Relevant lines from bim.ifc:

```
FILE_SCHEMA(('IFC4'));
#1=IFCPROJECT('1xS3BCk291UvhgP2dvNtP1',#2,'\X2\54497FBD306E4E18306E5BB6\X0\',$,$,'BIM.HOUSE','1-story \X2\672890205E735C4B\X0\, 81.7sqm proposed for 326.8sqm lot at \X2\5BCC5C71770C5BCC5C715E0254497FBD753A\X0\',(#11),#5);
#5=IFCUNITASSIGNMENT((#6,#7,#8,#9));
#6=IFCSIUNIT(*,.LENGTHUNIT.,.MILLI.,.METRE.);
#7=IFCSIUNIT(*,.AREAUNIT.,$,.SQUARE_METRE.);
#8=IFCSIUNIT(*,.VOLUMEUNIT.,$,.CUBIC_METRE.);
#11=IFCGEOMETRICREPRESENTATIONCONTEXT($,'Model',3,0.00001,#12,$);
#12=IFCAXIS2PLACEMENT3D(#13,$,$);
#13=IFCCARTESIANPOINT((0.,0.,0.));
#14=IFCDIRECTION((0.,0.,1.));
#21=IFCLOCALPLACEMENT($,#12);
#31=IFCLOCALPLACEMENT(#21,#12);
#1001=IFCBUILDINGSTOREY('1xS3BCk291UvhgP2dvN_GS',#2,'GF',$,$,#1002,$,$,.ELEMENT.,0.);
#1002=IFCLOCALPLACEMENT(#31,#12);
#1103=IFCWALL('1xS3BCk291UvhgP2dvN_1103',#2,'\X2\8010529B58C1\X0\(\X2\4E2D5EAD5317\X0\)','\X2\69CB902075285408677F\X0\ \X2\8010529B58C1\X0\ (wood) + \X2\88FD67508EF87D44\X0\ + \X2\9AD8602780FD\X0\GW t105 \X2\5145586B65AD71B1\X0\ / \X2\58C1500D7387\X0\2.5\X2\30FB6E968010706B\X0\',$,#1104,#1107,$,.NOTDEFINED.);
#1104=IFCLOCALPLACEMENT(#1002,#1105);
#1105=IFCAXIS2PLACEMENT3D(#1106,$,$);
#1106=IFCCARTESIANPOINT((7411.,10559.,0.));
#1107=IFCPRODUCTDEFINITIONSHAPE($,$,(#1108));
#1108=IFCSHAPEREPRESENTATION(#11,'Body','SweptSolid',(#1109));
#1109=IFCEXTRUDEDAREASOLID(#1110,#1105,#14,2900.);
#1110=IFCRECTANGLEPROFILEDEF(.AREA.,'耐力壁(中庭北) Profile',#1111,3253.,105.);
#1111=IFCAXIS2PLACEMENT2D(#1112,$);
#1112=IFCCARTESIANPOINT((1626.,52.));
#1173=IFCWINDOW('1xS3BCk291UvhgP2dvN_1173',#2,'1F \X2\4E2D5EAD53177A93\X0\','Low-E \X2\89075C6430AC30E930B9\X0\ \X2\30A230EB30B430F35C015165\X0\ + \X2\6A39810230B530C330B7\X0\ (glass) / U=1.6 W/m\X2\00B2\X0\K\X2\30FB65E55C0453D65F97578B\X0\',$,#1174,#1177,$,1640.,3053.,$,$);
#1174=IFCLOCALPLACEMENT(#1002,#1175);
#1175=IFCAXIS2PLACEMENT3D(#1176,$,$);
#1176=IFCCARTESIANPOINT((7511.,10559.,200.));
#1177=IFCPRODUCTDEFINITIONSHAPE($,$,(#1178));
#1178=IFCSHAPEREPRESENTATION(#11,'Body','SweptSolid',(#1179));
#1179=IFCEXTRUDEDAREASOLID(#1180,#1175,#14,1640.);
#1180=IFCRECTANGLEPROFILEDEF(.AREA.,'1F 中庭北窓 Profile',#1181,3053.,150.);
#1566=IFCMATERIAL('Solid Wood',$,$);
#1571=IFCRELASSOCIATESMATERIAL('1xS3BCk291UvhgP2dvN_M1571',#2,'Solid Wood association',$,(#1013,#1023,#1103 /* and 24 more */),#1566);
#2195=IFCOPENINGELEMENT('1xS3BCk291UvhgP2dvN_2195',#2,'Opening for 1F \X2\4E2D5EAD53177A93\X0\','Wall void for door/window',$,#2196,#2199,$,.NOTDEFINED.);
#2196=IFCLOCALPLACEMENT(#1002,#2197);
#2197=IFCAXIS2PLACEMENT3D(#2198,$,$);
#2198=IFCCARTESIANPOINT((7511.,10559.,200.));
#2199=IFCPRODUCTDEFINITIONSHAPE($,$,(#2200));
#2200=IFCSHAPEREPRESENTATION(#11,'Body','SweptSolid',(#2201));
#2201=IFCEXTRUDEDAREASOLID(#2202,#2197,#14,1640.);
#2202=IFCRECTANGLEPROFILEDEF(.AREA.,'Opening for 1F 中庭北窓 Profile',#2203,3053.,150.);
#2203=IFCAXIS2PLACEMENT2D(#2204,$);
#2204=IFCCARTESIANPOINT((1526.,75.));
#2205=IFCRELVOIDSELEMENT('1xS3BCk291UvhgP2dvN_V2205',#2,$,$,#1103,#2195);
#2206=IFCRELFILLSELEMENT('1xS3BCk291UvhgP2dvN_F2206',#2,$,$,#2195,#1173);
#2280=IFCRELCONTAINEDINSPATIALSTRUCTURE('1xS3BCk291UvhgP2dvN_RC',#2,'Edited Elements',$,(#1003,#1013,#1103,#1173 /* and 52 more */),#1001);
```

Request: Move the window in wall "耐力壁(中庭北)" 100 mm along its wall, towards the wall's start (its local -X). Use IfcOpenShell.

```python
import ifcopenshell
import ifcopenshell.api.geometry
import ifcopenshell.util.placement
import ifcopenshell.util.unit

model = ifcopenshell.open("bim.ifc")
unit_scale = ifcopenshell.util.unit.calculate_unit_scale(model)

window = model.by_guid("1xS3BCk291UvhgP2dvN_1173")
opening = window.FillsVoids[0].RelatingOpeningElement
wall = opening.VoidsElements[0].RelatingBuildingElement

wall_matrix = ifcopenshell.util.placement.get_local_placement(wall.ObjectPlacement)
shift = wall_matrix[:3, 0] * -0.1 / unit_scale
before = ifcopenshell.util.placement.get_local_placement(window.ObjectPlacement)[:3, 3].copy()

# The window is not placed relative to its opening, so move both.
for product in (opening, window):
    matrix = ifcopenshell.util.placement.get_local_placement(product.ObjectPlacement)
    matrix[:3, 3] += shift
    ifcopenshell.api.geometry.edit_object_placement(model, product=product, matrix=matrix, is_si=False)

after = ifcopenshell.util.placement.get_local_placement(window.ObjectPlacement)[:3, 3]
print("window moved by", (after - before).round(3) + 0.0)

model.write("bim-out.ifc")
```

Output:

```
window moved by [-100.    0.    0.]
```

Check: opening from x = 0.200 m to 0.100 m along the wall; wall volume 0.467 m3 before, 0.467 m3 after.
